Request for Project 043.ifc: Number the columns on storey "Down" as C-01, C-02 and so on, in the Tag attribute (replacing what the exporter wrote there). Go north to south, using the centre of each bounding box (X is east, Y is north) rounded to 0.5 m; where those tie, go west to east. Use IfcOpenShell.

First a look at what the model holds.

```python
import ifcopenshell
import ifcopenshell.util.element
import ifcopenshell.util.placement

model = ifcopenshell.open("Project 043.ifc")
print(model.schema)
storey = next(s for s in model.by_type("IfcBuildingStorey") if s.Name == "Down")
columns = [e for e in ifcopenshell.util.element.get_decomposition(storey) if e.is_a("IfcColumn")]
for e in sorted(columns, key=lambda e: e.id()):
    origin = ifcopenshell.util.placement.get_local_placement(e.ObjectPlacement)[:3, 3]
    print(e.id(), e.Tag, e.Name, origin.round(2) + 0.0, sep=" | ")
```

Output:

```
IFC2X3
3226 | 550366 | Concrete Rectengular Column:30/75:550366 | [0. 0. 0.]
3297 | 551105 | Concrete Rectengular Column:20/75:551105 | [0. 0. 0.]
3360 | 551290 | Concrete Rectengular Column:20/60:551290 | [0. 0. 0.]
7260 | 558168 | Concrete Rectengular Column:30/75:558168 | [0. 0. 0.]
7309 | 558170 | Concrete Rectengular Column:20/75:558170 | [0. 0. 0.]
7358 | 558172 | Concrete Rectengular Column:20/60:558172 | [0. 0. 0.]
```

```python
import ifcopenshell
import ifcopenshell.geom
import ifcopenshell.util.element
import ifcopenshell.util.shape

model = ifcopenshell.open("Project 043.ifc")
settings = ifcopenshell.geom.settings()
settings.set("use-world-coords", True)


def centre(element):
    shape = ifcopenshell.geom.create_shape(settings, element)
    return ifcopenshell.util.shape.get_bbox_centroid(shape.geometry)


storey = next(s for s in model.by_type("IfcBuildingStorey") if s.Name == "Down")
columns = [e for e in ifcopenshell.util.element.get_decomposition(storey) if e.is_a("IfcColumn")]

# Insertion points can sit at a corner or the storey origin, so sort by the geometry (in metres).
centres = {e: centre(e) for e in columns}
columns.sort(key=lambda e: (-round(centres[e][1] / 0.5), centres[e][0]))

for i, e in enumerate(columns, start=1):
    number = f"C-{i:02d}"
    e.Tag = number
    print(e.id(), number)

model.write("Project 043_updated.ifc")
```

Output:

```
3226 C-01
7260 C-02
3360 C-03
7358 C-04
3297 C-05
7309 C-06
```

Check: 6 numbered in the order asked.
